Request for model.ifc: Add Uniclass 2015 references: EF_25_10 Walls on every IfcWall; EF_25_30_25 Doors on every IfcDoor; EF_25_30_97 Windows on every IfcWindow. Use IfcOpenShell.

First a look at what the model holds.

```python
import ifcopenshell

model = ifcopenshell.open("model.ifc")
print(model.schema)
print("classifications:", [c.Name for c in model.by_type("IfcClassification")])
for ifc_class in ("IfcDoor", "IfcRoof", "IfcStair", "IfcWall", "IfcWindow"):
    print(ifc_class, len(model.by_type(ifc_class)))
```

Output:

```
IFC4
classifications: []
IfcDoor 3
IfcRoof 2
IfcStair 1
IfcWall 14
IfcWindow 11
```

```python
import ifcopenshell
import ifcopenshell.api.classification

model = ifcopenshell.open("model.ifc")

system = ifcopenshell.api.classification.add_classification(model, classification="Uniclass 2015")

codes = {
    "IfcWall": ("EF_25_10", "Walls"),
    "IfcDoor": ("EF_25_30_25", "Doors"),
    "IfcWindow": ("EF_25_30_97", "Windows"),
}
for ifc_class, (code, name) in codes.items():
    products = model.by_type(ifc_class)
    ifcopenshell.api.classification.add_reference(
        model, products=products, classification=system, identification=code, name=name
    )
    print(code, len(products))

model.write("model_rev.ifc")
```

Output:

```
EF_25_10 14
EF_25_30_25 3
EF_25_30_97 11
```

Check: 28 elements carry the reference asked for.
